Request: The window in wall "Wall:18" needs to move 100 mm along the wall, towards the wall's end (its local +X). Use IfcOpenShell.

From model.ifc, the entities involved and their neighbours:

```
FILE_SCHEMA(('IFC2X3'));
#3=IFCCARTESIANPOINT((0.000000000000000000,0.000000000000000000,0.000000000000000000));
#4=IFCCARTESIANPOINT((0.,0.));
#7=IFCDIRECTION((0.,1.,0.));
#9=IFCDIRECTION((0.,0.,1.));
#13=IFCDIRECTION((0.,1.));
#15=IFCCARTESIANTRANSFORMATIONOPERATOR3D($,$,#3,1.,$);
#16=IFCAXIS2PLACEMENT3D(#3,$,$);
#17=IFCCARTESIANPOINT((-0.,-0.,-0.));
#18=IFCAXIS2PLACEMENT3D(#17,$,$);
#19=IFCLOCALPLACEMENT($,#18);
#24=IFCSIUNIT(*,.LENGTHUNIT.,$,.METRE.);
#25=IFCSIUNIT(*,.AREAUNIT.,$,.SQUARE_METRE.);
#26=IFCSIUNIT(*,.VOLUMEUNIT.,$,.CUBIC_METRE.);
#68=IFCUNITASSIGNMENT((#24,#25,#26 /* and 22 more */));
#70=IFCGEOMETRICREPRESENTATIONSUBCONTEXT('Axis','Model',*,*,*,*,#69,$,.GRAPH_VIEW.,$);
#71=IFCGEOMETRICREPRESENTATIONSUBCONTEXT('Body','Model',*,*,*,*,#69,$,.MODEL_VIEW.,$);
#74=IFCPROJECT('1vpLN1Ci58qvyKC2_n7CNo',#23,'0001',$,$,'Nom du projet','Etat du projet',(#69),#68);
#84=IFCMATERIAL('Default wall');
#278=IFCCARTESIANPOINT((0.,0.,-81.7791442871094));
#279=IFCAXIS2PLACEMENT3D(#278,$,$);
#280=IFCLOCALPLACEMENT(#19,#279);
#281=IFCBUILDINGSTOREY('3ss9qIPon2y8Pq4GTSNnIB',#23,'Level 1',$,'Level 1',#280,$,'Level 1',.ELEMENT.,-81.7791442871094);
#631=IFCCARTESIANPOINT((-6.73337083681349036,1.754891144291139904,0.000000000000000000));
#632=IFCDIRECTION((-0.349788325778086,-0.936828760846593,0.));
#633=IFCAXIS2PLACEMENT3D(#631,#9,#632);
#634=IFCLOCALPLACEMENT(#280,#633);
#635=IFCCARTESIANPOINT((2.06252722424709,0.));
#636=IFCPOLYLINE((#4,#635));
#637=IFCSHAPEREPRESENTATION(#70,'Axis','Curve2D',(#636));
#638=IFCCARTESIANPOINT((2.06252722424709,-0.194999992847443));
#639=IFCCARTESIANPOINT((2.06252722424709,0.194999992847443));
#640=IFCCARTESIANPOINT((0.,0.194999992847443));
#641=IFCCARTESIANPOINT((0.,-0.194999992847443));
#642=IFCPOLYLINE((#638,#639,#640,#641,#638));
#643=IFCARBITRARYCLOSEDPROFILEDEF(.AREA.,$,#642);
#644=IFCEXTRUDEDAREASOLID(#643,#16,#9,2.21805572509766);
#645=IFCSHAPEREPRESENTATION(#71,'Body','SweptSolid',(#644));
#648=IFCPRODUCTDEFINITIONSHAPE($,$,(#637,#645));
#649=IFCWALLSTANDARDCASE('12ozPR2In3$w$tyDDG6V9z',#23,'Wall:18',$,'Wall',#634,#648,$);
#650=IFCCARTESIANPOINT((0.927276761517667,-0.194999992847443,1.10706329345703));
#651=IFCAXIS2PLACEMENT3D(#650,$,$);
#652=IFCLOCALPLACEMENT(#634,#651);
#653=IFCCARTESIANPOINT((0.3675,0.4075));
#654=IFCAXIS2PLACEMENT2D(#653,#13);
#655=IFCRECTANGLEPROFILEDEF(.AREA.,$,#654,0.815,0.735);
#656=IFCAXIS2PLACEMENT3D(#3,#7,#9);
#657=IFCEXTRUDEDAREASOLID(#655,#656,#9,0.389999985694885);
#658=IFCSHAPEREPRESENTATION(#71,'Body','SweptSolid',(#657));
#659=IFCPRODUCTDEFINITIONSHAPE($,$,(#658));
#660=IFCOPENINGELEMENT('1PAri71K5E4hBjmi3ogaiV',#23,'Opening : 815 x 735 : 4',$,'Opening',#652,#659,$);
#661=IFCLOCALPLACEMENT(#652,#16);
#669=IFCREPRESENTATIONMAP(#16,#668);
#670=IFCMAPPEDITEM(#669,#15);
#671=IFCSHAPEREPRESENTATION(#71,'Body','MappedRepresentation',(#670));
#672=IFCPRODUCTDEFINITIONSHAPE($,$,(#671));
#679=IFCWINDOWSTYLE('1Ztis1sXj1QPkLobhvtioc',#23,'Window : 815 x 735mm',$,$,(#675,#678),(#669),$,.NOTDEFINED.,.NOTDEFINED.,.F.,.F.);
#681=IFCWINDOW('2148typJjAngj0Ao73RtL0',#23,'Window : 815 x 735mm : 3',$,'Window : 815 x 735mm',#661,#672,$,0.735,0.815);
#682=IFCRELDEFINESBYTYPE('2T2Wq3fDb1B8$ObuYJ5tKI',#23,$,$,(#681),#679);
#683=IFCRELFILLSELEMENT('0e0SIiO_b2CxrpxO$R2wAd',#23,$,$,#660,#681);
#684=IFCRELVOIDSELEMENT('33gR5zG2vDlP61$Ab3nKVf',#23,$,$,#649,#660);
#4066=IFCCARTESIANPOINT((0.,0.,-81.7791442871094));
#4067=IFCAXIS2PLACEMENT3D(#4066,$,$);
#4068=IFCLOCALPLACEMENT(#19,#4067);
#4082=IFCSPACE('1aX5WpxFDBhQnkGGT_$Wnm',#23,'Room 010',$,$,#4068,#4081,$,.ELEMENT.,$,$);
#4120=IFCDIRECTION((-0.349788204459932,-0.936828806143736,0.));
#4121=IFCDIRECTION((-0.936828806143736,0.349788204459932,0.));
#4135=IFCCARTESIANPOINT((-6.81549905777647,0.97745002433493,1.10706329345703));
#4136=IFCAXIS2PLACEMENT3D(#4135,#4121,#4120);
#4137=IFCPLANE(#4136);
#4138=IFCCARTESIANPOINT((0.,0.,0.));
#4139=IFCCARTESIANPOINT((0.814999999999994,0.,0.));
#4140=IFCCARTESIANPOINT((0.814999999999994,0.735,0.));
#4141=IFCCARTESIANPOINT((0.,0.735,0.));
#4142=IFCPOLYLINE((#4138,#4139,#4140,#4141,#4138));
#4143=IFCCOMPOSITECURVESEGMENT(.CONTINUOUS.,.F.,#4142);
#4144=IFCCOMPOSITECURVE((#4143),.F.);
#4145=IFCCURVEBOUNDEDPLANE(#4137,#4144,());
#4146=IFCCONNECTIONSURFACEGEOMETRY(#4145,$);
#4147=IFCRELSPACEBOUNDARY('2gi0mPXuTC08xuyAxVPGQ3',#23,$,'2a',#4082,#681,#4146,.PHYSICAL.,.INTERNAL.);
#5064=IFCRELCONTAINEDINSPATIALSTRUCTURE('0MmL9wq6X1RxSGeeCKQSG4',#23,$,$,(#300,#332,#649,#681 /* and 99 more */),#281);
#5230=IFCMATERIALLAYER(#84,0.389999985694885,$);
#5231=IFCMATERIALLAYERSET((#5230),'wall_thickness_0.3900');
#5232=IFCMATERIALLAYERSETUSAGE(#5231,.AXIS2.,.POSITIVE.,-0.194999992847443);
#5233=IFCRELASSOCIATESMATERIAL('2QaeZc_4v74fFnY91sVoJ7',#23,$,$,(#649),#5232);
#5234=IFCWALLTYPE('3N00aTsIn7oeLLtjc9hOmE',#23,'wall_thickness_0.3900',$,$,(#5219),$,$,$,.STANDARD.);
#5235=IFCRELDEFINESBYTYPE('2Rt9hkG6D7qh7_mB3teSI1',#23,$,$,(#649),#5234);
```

```python
import numpy as np
import ifcopenshell
import ifcopenshell.api.geometry
import ifcopenshell.util.placement
import ifcopenshell.util.unit

model = ifcopenshell.open("model.ifc")
unit_scale = ifcopenshell.util.unit.calculate_unit_scale(model)

window = model.by_guid("2148typJjAngj0Ao73RtL0")
opening = window.FillsVoids[0].RelatingOpeningElement
wall = opening.VoidsElements[0].RelatingBuildingElement

wall_matrix = ifcopenshell.util.placement.get_local_placement(wall.ObjectPlacement)
shift = wall_matrix[:3, 0] * 0.1 / unit_scale
before = ifcopenshell.util.placement.get_local_placement(window.ObjectPlacement)[:3, 3].copy()

# The window is placed relative to its opening, so it follows when the opening moves.
matrix = ifcopenshell.util.placement.get_local_placement(opening.ObjectPlacement)
matrix[:3, 3] += shift
ifcopenshell.api.geometry.edit_object_placement(
    model, product=opening, matrix=matrix, is_si=False, should_transform_children=True
)

# Space boundary surfaces are stored in each space's coordinates; move them too.
for rel in window.ProvidesBoundaries:
    if not rel.ConnectionGeometry:
        continue
    surface = rel.ConnectionGeometry.SurfaceOnRelatingElement.BasisSurface
    space_matrix = ifcopenshell.util.placement.get_local_placement(rel.RelatingSpace.ObjectPlacement)
    point = np.array(surface.Position.Location.Coordinates) + space_matrix[:3, :3].T @ shift
    surface.Position = model.createIfcAxis2Placement3D(
        model.createIfcCartesianPoint(point.tolist()), surface.Position.Axis, surface.Position.RefDirection
    )

after = ifcopenshell.util.placement.get_local_placement(window.ObjectPlacement)[:3, 3]
print("window moved by", (after - before).round(3) + 0.0)

model.write("model_rev.ifc")
```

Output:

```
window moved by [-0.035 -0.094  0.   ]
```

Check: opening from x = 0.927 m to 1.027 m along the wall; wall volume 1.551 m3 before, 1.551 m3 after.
